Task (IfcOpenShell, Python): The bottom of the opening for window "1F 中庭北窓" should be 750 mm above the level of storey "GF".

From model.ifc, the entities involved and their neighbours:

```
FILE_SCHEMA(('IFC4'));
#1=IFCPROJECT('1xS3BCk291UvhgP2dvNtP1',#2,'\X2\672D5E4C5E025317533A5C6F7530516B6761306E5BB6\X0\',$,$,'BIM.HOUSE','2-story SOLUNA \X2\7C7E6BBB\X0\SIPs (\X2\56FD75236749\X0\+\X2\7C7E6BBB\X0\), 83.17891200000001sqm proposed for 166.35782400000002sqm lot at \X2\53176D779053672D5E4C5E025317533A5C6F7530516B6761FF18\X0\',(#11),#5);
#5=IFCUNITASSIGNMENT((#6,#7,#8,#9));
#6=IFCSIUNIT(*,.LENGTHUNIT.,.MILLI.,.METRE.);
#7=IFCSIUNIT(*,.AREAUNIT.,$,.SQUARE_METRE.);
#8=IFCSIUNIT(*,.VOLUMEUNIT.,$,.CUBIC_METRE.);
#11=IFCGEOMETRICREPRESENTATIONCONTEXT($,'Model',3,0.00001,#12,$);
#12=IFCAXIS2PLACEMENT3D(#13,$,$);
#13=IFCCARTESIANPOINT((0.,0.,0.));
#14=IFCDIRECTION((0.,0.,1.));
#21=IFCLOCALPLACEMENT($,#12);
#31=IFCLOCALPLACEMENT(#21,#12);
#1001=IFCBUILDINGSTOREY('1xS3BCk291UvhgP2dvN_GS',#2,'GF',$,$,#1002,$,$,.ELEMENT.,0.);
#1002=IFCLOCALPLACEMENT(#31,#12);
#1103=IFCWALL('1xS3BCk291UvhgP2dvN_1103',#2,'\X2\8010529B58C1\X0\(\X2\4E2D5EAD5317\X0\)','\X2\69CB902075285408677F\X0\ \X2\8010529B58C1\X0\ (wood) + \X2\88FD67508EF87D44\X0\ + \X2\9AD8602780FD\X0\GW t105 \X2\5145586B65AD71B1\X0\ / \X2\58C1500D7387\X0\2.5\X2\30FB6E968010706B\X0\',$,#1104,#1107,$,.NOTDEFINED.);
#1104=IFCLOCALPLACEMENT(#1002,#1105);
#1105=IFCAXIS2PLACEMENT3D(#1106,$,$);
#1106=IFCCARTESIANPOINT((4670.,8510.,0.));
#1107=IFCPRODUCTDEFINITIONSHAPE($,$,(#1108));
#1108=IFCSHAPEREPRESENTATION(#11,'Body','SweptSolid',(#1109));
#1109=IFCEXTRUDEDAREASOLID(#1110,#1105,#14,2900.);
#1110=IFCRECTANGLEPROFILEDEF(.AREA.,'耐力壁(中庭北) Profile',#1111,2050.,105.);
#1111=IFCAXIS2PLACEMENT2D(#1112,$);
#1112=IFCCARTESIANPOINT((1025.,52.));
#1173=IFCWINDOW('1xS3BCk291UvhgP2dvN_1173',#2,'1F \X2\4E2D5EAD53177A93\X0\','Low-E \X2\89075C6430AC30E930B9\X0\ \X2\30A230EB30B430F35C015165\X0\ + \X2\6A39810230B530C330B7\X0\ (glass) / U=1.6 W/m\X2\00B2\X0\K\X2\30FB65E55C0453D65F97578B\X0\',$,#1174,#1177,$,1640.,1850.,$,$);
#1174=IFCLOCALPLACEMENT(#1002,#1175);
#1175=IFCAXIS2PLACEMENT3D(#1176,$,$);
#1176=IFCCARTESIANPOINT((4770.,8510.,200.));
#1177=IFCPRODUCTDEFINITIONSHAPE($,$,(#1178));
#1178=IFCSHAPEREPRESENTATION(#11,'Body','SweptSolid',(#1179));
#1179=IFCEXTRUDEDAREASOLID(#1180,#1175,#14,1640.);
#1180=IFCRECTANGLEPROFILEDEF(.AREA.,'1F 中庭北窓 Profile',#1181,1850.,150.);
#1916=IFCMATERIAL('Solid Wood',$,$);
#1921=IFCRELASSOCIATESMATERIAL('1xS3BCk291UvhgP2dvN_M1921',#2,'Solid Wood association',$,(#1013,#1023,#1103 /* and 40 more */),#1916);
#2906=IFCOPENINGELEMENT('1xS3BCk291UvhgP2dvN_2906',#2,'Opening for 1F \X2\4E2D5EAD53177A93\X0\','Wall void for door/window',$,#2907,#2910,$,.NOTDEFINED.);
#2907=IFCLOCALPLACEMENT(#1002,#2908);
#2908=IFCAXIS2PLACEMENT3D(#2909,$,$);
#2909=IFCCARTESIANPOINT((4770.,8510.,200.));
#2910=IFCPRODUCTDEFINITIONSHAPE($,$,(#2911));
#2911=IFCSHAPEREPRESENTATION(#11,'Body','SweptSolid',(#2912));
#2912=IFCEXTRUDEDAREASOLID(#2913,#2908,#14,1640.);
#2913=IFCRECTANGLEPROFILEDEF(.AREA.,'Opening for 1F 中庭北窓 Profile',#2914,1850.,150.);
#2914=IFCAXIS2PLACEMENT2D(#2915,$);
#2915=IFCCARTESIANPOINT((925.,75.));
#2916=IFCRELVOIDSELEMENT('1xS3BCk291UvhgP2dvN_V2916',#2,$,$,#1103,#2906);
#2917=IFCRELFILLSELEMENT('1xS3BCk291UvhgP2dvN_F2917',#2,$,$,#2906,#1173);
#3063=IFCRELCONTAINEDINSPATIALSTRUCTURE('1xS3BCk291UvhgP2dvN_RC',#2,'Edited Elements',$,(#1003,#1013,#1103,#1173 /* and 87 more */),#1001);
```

```python
import numpy as np
import ifcopenshell
import ifcopenshell.api.geometry
import ifcopenshell.geom
import ifcopenshell.util.element
import ifcopenshell.util.placement
import ifcopenshell.util.shape
import ifcopenshell.util.unit

model = ifcopenshell.open("model.ifc")
unit_scale = ifcopenshell.util.unit.calculate_unit_scale(model)

window = model.by_id(1173)
opening = window.FillsVoids[0].RelatingOpeningElement
storey = ifcopenshell.util.element.get_container(window, ifc_class="IfcBuildingStorey")
level = ifcopenshell.util.placement.get_local_placement(storey.ObjectPlacement)[2, 3]

# The opening's origin need not be at the sill, so measure its lowest point.
shape = ifcopenshell.geom.create_shape(ifcopenshell.geom.settings(), opening)
bottom = ifcopenshell.util.shape.get_shape_bottom_elevation(shape, shape.geometry) / unit_scale
dz = level + 0.75 / unit_scale - bottom

shift = np.array([0.0, 0.0, dz])
# The window is not placed relative to its opening, so move both.
for product in (opening, window):
    matrix = ifcopenshell.util.placement.get_local_placement(product.ObjectPlacement)
    matrix[:3, 3] += shift
    ifcopenshell.api.geometry.edit_object_placement(model, product=product, matrix=matrix, is_si=False)

print(f"moved by {dz * unit_scale:+.3f} m")

model.write("model_rev.ifc")
```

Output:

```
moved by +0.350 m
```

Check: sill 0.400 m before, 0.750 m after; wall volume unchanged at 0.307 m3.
